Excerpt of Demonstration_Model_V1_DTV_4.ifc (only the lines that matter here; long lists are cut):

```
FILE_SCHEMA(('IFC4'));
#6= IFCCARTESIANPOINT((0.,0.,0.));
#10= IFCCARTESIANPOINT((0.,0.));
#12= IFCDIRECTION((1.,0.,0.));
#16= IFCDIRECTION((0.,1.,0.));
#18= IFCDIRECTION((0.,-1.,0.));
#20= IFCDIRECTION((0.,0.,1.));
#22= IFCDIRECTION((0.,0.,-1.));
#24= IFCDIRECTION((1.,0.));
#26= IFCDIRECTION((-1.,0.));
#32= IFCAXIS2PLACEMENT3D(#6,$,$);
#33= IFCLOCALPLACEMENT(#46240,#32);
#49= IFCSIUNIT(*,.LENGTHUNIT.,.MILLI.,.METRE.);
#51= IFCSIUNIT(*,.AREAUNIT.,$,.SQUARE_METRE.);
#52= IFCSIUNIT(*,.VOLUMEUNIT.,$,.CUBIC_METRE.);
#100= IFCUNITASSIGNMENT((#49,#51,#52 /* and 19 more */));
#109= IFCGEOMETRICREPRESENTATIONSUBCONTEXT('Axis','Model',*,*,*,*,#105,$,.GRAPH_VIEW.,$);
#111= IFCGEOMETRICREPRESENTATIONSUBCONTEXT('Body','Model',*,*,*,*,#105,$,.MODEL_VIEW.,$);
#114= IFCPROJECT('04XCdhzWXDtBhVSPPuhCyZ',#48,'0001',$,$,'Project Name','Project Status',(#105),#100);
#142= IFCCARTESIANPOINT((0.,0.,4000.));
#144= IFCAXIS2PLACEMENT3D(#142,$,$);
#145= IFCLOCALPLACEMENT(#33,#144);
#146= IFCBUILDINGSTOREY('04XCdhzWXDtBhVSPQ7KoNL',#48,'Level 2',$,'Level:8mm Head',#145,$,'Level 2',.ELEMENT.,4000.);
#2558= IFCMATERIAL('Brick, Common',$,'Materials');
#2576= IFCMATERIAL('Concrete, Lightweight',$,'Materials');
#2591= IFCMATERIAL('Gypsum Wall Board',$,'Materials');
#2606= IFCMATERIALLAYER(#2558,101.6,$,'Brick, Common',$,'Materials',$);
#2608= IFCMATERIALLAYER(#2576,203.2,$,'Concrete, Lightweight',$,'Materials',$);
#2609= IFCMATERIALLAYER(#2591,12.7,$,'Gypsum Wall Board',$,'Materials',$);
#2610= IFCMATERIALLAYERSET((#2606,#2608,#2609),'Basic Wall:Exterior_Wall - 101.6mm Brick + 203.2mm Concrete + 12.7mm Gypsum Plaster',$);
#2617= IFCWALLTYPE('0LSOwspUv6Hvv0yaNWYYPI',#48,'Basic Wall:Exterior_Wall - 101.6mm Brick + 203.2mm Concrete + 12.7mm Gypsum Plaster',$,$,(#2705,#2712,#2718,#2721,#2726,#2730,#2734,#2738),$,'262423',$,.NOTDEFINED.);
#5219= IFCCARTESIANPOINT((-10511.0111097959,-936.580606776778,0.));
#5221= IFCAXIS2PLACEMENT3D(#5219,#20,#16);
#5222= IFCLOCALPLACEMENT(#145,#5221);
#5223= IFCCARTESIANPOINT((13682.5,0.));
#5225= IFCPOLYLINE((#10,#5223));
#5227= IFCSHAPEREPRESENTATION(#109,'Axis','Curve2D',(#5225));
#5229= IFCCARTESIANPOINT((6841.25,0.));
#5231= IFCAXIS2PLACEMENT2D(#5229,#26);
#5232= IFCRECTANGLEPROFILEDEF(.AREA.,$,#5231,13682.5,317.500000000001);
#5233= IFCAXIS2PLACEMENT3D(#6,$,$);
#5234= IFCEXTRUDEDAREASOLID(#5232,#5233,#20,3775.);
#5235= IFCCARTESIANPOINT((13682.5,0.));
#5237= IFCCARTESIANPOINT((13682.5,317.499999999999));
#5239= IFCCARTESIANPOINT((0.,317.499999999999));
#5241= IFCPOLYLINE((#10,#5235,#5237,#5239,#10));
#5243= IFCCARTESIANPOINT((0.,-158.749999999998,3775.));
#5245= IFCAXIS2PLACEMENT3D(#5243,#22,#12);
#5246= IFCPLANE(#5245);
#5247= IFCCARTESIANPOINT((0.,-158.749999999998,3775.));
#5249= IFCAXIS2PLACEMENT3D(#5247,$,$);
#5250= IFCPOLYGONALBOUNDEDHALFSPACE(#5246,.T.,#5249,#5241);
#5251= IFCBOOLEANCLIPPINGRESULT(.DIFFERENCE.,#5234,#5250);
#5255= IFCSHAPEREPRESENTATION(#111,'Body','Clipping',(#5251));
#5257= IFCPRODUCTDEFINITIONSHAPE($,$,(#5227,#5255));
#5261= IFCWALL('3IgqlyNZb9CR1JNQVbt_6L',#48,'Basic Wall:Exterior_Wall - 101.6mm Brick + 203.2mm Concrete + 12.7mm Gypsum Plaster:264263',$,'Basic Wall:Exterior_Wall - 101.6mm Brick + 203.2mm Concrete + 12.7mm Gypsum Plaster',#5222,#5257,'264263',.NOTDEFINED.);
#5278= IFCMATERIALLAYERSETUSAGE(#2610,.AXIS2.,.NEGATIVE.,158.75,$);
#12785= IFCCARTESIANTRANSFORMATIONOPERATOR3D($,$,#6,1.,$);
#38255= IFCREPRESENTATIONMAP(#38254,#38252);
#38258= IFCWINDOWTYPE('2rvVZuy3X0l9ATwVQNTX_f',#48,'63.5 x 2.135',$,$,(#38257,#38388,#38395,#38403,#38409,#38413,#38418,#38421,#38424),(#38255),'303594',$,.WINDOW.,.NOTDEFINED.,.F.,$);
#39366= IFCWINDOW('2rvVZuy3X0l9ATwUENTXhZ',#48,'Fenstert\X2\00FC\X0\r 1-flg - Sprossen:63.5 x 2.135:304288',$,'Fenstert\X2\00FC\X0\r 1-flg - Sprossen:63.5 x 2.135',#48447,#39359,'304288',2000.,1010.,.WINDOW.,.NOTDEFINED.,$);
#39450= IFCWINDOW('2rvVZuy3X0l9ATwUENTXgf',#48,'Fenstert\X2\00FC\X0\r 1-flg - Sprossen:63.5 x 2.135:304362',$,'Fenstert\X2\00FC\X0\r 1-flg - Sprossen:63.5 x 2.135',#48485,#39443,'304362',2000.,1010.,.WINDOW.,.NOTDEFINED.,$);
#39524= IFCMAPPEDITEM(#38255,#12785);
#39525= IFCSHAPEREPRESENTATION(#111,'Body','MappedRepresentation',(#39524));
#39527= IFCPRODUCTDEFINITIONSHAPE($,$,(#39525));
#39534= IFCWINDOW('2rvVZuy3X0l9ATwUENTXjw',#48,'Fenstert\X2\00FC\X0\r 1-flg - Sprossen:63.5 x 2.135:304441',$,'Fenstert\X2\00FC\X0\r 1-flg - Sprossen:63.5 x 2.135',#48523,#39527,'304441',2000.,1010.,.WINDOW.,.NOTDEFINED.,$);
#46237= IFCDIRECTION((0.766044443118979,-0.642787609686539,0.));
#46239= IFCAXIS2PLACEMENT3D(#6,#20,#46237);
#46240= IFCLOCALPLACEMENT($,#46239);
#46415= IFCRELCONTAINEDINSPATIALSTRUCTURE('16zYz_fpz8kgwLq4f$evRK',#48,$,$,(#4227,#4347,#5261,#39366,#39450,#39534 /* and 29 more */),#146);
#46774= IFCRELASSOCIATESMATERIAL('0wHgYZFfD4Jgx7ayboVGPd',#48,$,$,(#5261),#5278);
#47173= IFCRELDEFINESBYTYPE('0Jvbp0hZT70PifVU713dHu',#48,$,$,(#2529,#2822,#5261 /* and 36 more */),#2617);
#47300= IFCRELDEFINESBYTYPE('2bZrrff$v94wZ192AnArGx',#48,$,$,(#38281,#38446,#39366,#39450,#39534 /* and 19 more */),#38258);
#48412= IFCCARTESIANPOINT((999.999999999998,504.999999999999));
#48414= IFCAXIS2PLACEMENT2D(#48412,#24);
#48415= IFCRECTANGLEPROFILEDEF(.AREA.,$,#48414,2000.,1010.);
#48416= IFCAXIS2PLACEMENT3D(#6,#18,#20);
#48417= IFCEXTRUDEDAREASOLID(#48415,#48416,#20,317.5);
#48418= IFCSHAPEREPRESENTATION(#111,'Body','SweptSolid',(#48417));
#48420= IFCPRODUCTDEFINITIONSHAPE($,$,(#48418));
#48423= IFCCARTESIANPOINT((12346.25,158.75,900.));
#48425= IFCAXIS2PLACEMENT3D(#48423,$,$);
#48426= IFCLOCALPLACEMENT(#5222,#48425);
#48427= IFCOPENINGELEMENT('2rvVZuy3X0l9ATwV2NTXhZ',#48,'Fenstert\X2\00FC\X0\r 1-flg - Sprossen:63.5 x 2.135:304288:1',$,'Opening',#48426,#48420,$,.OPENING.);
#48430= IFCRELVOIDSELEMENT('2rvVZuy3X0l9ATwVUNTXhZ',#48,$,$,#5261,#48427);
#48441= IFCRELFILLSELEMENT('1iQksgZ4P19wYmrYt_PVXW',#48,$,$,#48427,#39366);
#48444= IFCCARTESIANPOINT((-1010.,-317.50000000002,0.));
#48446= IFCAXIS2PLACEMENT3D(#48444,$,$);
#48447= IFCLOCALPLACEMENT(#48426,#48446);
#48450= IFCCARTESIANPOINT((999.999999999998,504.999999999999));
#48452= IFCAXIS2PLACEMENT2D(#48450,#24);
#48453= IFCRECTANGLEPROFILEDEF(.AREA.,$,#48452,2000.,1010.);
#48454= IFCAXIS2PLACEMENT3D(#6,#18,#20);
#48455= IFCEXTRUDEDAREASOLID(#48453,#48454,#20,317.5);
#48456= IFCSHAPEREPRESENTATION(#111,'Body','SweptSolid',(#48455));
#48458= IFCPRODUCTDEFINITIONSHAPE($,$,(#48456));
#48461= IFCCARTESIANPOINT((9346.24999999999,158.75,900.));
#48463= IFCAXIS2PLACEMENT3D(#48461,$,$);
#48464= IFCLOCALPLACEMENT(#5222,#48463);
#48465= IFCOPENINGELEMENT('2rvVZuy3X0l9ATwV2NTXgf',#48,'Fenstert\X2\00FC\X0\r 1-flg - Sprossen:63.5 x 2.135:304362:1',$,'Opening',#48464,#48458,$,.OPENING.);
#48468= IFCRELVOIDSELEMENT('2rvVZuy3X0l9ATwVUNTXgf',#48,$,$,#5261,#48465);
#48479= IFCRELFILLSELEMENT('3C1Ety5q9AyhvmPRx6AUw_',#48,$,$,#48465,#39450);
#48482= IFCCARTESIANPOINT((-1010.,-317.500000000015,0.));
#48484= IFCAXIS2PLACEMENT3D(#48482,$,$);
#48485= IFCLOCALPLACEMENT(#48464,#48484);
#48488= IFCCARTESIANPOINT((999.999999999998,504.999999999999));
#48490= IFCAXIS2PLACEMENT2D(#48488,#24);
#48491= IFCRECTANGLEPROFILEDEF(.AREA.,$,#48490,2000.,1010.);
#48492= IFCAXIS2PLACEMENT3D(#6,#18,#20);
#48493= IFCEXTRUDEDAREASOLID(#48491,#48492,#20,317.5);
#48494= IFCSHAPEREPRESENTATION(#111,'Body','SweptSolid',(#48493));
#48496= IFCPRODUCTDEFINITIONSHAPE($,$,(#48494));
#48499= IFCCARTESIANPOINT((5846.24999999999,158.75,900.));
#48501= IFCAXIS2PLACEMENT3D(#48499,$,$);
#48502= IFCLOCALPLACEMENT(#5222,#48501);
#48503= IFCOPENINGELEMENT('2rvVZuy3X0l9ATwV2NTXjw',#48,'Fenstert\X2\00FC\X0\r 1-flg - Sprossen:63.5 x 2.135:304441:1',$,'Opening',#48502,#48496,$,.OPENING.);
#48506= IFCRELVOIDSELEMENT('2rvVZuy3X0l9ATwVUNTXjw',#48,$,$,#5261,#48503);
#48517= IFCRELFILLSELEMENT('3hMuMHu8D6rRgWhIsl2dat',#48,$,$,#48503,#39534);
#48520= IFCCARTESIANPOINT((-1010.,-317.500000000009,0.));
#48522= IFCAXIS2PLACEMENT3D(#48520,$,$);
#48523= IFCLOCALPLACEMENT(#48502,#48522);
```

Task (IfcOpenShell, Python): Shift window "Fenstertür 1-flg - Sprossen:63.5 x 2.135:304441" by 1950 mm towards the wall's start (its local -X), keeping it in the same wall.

```python
import ifcopenshell
import ifcopenshell.api.geometry
import ifcopenshell.util.placement
import ifcopenshell.util.unit

model = ifcopenshell.open("Demonstration_Model_V1_DTV_4.ifc")
unit_scale = ifcopenshell.util.unit.calculate_unit_scale(model)

window = model.by_guid("2rvVZuy3X0l9ATwUENTXjw")
opening = window.FillsVoids[0].RelatingOpeningElement
wall = opening.VoidsElements[0].RelatingBuildingElement

wall_matrix = ifcopenshell.util.placement.get_local_placement(wall.ObjectPlacement)
shift = wall_matrix[:3, 0] * -1.95 / unit_scale
before = ifcopenshell.util.placement.get_local_placement(window.ObjectPlacement)[:3, 3].copy()

# The window is placed relative to its opening, so it follows when the opening moves.
matrix = ifcopenshell.util.placement.get_local_placement(opening.ObjectPlacement)
matrix[:3, 3] += shift
ifcopenshell.api.geometry.edit_object_placement(
    model, product=opening, matrix=matrix, is_si=False, should_transform_children=True
)

after = ifcopenshell.util.placement.get_local_placement(window.ObjectPlacement)[:3, 3]
print("window moved by", (after - before).round(3) + 0.0)

model.write("Demonstration_Model_V1_DTV_4_rev.ifc")
```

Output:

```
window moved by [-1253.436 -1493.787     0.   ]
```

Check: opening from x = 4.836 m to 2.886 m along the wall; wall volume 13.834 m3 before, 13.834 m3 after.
